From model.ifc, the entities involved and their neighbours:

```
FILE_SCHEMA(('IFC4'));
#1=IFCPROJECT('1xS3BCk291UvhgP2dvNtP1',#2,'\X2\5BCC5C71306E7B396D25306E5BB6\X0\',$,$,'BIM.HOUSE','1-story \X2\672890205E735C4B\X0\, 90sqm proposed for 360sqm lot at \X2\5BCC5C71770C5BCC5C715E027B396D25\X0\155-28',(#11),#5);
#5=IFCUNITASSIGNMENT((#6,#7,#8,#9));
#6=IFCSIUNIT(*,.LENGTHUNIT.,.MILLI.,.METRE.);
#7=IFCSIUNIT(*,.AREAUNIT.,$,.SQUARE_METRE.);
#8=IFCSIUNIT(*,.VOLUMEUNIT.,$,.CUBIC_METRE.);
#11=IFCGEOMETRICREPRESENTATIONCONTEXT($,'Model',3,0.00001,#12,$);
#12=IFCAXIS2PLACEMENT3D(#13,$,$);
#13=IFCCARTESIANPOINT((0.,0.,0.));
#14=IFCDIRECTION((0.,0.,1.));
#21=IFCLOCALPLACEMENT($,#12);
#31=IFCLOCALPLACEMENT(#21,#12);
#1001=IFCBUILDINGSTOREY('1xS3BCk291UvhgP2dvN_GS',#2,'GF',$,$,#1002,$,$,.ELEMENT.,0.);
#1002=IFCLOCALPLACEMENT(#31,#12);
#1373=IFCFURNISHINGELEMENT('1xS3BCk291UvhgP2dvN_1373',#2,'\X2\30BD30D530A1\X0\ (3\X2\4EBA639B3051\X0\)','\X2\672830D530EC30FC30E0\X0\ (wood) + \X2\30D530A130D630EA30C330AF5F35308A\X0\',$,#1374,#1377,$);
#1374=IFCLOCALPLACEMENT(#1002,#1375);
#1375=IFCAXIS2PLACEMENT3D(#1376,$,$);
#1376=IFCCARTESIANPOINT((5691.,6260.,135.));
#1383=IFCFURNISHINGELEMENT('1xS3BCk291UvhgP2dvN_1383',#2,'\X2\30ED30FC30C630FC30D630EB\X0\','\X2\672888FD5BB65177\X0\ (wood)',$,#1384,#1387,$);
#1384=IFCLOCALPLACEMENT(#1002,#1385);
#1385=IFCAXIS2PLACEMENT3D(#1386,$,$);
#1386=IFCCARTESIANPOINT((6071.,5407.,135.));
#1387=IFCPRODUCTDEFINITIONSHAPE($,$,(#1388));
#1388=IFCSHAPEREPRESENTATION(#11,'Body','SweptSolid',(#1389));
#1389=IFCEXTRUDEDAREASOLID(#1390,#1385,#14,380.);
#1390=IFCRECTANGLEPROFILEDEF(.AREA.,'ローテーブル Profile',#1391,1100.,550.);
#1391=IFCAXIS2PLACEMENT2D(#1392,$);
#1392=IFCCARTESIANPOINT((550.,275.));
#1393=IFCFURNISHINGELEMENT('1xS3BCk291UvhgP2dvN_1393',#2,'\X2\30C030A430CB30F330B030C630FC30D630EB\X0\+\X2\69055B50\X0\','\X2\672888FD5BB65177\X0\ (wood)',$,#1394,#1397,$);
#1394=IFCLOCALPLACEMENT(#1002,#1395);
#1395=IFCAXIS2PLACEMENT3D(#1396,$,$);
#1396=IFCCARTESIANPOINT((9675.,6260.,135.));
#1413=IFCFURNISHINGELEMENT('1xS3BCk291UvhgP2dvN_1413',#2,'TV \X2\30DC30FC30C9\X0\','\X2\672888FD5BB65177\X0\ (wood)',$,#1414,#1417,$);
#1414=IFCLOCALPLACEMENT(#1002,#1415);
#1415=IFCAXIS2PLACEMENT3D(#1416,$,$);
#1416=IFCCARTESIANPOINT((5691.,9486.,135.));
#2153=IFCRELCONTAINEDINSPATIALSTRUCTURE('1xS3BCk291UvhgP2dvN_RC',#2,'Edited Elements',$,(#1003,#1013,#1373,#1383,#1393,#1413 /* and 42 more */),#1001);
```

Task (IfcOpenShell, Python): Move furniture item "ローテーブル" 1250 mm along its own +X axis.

```python
import ifcopenshell
import ifcopenshell.api.geometry
import ifcopenshell.util.placement
import ifcopenshell.util.unit

model = ifcopenshell.open("model.ifc")
unit_scale = ifcopenshell.util.unit.calculate_unit_scale(model)

item = model.by_guid("1xS3BCk291UvhgP2dvN_1383")
matrix = ifcopenshell.util.placement.get_local_placement(item.ObjectPlacement)
matrix[:3, 3] += matrix[:3, 0] * 1.25 / unit_scale
ifcopenshell.api.geometry.edit_object_placement(model, product=item, matrix=matrix, is_si=False)

print(ifcopenshell.util.placement.get_local_placement(item.ObjectPlacement).round(3) + 0.0)

model.write("model_updated.ifc")
```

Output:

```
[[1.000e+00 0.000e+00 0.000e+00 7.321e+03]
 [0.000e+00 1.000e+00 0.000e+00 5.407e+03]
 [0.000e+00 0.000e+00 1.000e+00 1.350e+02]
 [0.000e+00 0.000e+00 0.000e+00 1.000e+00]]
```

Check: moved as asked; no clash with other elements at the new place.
